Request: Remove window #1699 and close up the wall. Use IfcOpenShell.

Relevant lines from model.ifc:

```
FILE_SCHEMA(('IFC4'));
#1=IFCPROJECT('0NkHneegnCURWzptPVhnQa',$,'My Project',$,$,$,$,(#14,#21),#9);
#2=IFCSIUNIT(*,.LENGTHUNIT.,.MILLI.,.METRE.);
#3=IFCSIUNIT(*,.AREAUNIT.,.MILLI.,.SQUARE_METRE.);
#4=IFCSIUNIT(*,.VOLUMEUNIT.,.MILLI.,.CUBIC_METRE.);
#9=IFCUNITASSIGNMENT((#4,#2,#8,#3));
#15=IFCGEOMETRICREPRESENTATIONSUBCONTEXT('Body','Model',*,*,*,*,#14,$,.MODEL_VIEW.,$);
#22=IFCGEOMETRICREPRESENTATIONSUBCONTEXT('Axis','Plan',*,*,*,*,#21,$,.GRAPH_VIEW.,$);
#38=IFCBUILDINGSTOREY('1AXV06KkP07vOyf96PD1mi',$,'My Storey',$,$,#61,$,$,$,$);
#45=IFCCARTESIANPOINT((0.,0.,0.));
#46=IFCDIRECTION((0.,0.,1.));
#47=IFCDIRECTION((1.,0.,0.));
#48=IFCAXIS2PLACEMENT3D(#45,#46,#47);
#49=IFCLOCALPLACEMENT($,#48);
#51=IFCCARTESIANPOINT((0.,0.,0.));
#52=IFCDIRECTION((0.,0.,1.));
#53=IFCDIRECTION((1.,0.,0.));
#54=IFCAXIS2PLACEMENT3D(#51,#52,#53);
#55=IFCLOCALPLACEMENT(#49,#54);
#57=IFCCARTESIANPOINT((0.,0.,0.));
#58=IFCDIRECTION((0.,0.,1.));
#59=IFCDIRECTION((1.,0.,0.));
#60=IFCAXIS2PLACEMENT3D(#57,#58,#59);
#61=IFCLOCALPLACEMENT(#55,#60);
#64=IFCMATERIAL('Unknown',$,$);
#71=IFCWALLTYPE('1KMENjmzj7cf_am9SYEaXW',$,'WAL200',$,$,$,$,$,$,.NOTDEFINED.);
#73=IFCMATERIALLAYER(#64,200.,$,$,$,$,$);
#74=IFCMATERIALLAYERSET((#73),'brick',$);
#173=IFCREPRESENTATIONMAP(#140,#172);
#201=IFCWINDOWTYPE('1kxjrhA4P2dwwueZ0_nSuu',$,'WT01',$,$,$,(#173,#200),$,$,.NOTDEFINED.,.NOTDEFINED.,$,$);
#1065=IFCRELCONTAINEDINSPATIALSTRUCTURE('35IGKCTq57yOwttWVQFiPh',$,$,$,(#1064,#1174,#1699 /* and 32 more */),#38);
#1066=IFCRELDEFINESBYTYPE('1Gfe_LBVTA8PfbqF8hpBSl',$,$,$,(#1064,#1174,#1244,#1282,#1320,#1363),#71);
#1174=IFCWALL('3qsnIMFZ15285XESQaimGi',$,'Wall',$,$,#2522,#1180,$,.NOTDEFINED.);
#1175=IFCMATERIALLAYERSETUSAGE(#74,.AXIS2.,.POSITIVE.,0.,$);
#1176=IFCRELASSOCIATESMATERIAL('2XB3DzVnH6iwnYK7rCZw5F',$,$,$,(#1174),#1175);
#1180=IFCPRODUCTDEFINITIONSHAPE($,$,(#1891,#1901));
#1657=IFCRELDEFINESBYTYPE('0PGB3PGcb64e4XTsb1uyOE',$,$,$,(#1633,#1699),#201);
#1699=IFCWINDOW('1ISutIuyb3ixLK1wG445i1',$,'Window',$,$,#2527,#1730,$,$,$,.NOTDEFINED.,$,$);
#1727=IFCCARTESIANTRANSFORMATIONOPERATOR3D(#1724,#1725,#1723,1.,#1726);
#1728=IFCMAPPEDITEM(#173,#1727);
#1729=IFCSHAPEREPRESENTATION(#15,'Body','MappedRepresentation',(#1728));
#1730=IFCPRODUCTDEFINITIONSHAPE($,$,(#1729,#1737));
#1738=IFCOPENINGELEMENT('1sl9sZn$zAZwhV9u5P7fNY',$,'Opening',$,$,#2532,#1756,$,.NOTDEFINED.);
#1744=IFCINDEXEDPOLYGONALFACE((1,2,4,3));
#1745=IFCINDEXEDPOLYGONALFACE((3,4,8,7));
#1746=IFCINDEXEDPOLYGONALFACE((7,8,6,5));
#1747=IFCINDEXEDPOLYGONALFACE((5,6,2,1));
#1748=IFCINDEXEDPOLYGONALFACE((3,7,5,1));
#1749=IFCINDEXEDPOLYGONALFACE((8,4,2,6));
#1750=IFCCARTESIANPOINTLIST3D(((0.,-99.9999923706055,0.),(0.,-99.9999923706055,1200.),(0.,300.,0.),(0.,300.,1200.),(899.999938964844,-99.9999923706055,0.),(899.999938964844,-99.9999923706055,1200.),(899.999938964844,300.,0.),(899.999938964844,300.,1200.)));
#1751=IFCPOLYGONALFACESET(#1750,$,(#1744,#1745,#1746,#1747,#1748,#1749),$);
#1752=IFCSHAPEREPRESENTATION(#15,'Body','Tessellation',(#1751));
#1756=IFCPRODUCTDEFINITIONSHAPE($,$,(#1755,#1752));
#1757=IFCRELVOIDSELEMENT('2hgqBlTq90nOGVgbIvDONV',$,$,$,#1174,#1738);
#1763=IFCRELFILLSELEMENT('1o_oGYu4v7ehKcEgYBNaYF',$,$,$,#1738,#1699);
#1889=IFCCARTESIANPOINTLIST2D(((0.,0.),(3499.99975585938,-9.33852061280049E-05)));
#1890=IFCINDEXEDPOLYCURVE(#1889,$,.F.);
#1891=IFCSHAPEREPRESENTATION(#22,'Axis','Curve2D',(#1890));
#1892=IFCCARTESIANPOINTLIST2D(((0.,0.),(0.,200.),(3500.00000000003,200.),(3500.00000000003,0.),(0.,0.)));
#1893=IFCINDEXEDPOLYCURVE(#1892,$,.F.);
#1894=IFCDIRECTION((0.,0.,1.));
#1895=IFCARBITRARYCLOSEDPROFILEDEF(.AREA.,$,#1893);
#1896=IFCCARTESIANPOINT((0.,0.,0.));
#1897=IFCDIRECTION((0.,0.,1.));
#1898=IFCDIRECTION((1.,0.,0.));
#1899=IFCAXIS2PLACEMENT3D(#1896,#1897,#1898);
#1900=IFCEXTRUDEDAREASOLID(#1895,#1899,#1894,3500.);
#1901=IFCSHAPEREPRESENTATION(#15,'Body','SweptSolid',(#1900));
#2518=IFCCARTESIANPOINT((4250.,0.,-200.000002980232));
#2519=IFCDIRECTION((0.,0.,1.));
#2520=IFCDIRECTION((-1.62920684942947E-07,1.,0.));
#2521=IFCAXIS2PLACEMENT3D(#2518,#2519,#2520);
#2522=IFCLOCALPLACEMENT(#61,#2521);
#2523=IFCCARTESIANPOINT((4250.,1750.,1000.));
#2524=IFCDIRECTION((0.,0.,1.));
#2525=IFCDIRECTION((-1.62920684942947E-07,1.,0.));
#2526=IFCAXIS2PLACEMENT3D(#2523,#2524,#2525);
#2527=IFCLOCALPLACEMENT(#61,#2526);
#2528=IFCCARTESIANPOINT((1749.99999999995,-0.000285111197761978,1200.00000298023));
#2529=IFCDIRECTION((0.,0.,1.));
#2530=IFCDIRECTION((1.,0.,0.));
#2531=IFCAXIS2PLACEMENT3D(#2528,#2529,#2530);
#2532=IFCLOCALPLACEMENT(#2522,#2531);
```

```python
import ifcopenshell
import ifcopenshell.api.feature
import ifcopenshell.api.root
import ifcopenshell.geom
import ifcopenshell.util.shape

model = ifcopenshell.open("model.ifc")
settings = ifcopenshell.geom.settings()


def volume(element):
    """Net volume in cubic metres, openings subtracted."""
    shape = ifcopenshell.geom.create_shape(settings, element)
    return ifcopenshell.util.shape.get_volume(shape.geometry)


window = model.by_id(1699)
opening = window.FillsVoids[0].RelatingOpeningElement
wall = opening.VoidsElements[0].RelatingBuildingElement
before = volume(wall)

ifcopenshell.api.root.remove_product(model, product=window)
ifcopenshell.api.feature.remove_feature(model, feature=opening)

after = volume(wall)

print(f"wall volume {before:.3f} -> {after:.3f} m3")

model.write("model_updated.ifc")
```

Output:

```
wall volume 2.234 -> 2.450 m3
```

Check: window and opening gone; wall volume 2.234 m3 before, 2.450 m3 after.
